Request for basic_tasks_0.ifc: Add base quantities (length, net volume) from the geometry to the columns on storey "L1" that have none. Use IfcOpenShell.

First a look at what the model holds.

```python
import ifcopenshell
import ifcopenshell.util.element
import ifcopenshell.util.unit

model = ifcopenshell.open("basic_tasks_0.ifc")
print(model.schema)
for unit_type in ("LENGTHUNIT", "AREAUNIT", "VOLUMEUNIT"):
    print(unit_type, ifcopenshell.util.unit.calculate_unit_scale(model, unit_type))
storey = next(s for s in model.by_type("IfcBuildingStorey") if s.Name == "L1")
columns = [e for e in ifcopenshell.util.element.get_decomposition(storey) if e.is_a("IfcColumn")]
for e in sorted(columns, key=lambda e: e.id()):
    print(e.id(), e.is_a(), e.Name, list(ifcopenshell.util.element.get_psets(e, qtos_only=True)), sep=" | ")
```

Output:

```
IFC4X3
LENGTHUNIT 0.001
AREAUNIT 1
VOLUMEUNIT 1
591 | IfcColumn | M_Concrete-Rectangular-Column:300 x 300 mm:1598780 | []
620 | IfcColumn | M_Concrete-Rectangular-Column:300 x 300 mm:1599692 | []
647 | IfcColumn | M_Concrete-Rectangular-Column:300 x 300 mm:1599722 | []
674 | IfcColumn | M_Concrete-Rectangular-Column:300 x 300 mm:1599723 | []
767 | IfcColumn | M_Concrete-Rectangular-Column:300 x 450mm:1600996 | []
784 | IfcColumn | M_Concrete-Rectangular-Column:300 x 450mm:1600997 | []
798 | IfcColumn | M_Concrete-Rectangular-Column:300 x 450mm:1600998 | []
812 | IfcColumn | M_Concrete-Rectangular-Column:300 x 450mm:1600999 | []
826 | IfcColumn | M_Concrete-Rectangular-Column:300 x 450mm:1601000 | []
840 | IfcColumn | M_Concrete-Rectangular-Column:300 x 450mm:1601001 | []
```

```python
import ifcopenshell
import ifcopenshell.api.pset
import ifcopenshell.geom
import ifcopenshell.util.element
import ifcopenshell.util.shape
import ifcopenshell.util.unit

model = ifcopenshell.open("basic_tasks_0.ifc")
unit_scale = ifcopenshell.util.unit.calculate_unit_scale(model)
volume_scale = ifcopenshell.util.unit.calculate_unit_scale(model, "VOLUMEUNIT")
settings = ifcopenshell.geom.settings()

storey = next(s for s in model.by_type("IfcBuildingStorey") if s.Name == "L1")
columns = [e for e in ifcopenshell.util.element.get_decomposition(storey) if e.is_a("IfcColumn")]

for e in sorted(columns, key=lambda e: e.id()):
    if ifcopenshell.util.element.get_psets(e, qtos_only=True, should_inherit=False):
        continue
    # Geometry comes back in metres, in the element's own axes.
    shape = ifcopenshell.geom.create_shape(settings, e)
    values = {
        "Length": ifcopenshell.util.shape.get_z(shape.geometry) / unit_scale,
        "NetVolume": ifcopenshell.util.shape.get_volume(shape.geometry) / volume_scale,
    }
    qto = ifcopenshell.api.pset.add_qto(model, product=e, name="Qto_ColumnBaseQuantities")
    ifcopenshell.api.pset.edit_qto(model, qto=qto, properties=values)
    print(e.id(), {k: round(v, 3) for k, v in values.items()})

model.write("basic_tasks_0-out.ifc")
```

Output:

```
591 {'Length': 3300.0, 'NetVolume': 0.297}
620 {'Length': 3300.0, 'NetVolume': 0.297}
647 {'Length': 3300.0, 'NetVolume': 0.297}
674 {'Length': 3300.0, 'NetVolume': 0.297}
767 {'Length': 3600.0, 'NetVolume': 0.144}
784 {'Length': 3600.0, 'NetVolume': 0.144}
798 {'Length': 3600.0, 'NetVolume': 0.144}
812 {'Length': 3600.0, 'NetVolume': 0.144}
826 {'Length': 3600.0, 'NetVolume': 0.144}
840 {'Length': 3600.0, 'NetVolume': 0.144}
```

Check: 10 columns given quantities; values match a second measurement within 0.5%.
